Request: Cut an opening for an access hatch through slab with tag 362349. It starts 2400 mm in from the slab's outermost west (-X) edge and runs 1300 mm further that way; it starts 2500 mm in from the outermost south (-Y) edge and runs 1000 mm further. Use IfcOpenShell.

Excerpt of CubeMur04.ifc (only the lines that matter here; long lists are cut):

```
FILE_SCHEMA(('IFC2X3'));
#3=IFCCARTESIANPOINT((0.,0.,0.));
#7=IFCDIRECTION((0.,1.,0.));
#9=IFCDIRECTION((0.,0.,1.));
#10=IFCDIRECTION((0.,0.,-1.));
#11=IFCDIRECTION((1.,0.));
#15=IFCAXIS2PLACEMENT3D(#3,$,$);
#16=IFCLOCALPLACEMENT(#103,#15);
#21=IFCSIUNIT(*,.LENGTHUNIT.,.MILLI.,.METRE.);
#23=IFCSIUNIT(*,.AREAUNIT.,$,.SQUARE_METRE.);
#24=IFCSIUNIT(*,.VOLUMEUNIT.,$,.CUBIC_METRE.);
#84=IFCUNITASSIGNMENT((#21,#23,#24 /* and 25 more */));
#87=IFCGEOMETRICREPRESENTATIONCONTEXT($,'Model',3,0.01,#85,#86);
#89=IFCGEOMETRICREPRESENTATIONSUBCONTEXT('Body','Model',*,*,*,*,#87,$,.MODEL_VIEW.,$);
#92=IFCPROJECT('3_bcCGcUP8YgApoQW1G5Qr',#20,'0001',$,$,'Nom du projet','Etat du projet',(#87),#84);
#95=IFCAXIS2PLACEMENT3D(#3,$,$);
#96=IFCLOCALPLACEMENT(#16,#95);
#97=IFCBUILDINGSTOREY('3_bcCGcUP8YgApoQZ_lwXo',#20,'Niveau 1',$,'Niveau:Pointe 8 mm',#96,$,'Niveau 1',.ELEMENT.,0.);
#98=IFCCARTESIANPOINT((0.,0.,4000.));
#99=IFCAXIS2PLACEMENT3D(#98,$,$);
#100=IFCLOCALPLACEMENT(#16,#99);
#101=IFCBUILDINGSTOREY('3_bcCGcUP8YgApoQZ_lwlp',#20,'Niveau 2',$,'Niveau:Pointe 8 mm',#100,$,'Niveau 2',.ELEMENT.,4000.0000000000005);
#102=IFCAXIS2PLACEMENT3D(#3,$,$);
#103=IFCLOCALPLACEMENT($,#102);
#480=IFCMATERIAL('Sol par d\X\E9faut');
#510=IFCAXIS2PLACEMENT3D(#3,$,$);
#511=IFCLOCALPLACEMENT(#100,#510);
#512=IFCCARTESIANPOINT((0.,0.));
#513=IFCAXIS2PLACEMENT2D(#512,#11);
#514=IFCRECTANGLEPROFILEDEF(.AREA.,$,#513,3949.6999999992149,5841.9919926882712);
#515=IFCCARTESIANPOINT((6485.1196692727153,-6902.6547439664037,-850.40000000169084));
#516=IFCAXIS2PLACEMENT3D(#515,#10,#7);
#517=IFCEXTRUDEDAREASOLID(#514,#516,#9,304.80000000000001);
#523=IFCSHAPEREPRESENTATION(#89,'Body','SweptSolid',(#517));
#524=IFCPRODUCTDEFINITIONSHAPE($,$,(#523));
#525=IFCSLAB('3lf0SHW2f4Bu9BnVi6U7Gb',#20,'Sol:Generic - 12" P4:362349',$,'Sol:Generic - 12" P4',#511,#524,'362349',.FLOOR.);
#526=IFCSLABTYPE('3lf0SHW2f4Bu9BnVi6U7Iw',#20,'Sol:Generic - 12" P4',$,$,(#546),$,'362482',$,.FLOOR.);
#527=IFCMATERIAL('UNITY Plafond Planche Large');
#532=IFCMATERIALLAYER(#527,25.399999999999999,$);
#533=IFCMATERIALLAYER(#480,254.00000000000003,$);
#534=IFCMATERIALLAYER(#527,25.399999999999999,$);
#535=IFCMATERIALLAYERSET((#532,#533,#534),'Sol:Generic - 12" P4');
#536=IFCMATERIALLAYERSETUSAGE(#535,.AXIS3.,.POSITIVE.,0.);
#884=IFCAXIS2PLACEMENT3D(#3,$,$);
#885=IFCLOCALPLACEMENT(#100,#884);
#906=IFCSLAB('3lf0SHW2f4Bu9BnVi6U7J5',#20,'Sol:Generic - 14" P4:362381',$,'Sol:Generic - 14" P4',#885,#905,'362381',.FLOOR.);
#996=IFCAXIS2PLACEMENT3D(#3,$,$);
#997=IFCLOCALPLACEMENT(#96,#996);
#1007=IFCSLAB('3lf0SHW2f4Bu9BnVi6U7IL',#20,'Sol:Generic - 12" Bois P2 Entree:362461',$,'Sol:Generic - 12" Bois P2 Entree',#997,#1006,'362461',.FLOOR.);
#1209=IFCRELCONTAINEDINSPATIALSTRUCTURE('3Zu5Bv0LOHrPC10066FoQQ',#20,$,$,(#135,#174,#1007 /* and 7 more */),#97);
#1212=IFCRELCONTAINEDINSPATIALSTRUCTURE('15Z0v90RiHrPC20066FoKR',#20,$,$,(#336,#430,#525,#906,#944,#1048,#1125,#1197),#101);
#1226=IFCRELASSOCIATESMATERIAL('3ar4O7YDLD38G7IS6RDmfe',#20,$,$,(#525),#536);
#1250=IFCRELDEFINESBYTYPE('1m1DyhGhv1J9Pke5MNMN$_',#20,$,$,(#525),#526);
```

```python
import numpy as np
import ifcopenshell
import ifcopenshell.api.feature
import ifcopenshell.api.geometry
import ifcopenshell.api.root
import ifcopenshell.geom
import ifcopenshell.util.placement
import ifcopenshell.util.representation
import ifcopenshell.util.shape
import ifcopenshell.util.unit

model = ifcopenshell.open("CubeMur04.ifc")
unit_scale = ifcopenshell.util.unit.calculate_unit_scale(model)
settings = ifcopenshell.geom.settings()


def volume(element):
    """Net volume in cubic metres, openings subtracted."""
    shape = ifcopenshell.geom.create_shape(settings, element)
    return ifcopenshell.util.shape.get_volume(shape.geometry)


slab = model.by_guid("3lf0SHW2f4Bu9BnVi6U7Gb")
before = volume(slab)

# Extent in the slab's own axes, in metres. The edges named are its -X and -Y sides.
slab_shape = ifcopenshell.geom.create_shape(settings, slab)
vertices = ifcopenshell.util.shape.get_vertices(slab_shape.geometry)
x_min, y_min, bottom = vertices.min(axis=0)
top = vertices[:, 2].max()

opening = ifcopenshell.api.root.create_entity(model, ifc_class="IfcOpeningElement", name="Access hatch opening")
context = ifcopenshell.util.representation.get_context(model, "Model", "Body", "MODEL_VIEW")
width, depth = 1.3, 1
outline = [(0.0, 0.0), (width, 0.0), (width, depth), (0.0, depth), (0.0, 0.0)]
# Overshoot both faces by 50 mm so the cut is clean.
shape = ifcopenshell.api.geometry.add_slab_representation(
    model, context=context, depth=top - bottom + 0.1, polyline=outline
)
ifcopenshell.api.geometry.assign_representation(model, product=opening, representation=shape)

matrix = ifcopenshell.util.placement.get_local_placement(slab.ObjectPlacement)
matrix[:, 3] = matrix @ np.append(np.array([x_min + 2.4, y_min + 2.5, bottom - 0.05]) / unit_scale, 1.0)
ifcopenshell.api.geometry.edit_object_placement(model, product=opening, matrix=matrix, is_si=False)
ifcopenshell.api.feature.add_feature(model, feature=opening, element=slab)

after = volume(slab)

print(f"slab volume {before:.3f} -> {after:.3f} m3")

model.write("CubeMur04-out.ifc")
```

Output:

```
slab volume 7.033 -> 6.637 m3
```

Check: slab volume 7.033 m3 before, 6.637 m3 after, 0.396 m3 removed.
